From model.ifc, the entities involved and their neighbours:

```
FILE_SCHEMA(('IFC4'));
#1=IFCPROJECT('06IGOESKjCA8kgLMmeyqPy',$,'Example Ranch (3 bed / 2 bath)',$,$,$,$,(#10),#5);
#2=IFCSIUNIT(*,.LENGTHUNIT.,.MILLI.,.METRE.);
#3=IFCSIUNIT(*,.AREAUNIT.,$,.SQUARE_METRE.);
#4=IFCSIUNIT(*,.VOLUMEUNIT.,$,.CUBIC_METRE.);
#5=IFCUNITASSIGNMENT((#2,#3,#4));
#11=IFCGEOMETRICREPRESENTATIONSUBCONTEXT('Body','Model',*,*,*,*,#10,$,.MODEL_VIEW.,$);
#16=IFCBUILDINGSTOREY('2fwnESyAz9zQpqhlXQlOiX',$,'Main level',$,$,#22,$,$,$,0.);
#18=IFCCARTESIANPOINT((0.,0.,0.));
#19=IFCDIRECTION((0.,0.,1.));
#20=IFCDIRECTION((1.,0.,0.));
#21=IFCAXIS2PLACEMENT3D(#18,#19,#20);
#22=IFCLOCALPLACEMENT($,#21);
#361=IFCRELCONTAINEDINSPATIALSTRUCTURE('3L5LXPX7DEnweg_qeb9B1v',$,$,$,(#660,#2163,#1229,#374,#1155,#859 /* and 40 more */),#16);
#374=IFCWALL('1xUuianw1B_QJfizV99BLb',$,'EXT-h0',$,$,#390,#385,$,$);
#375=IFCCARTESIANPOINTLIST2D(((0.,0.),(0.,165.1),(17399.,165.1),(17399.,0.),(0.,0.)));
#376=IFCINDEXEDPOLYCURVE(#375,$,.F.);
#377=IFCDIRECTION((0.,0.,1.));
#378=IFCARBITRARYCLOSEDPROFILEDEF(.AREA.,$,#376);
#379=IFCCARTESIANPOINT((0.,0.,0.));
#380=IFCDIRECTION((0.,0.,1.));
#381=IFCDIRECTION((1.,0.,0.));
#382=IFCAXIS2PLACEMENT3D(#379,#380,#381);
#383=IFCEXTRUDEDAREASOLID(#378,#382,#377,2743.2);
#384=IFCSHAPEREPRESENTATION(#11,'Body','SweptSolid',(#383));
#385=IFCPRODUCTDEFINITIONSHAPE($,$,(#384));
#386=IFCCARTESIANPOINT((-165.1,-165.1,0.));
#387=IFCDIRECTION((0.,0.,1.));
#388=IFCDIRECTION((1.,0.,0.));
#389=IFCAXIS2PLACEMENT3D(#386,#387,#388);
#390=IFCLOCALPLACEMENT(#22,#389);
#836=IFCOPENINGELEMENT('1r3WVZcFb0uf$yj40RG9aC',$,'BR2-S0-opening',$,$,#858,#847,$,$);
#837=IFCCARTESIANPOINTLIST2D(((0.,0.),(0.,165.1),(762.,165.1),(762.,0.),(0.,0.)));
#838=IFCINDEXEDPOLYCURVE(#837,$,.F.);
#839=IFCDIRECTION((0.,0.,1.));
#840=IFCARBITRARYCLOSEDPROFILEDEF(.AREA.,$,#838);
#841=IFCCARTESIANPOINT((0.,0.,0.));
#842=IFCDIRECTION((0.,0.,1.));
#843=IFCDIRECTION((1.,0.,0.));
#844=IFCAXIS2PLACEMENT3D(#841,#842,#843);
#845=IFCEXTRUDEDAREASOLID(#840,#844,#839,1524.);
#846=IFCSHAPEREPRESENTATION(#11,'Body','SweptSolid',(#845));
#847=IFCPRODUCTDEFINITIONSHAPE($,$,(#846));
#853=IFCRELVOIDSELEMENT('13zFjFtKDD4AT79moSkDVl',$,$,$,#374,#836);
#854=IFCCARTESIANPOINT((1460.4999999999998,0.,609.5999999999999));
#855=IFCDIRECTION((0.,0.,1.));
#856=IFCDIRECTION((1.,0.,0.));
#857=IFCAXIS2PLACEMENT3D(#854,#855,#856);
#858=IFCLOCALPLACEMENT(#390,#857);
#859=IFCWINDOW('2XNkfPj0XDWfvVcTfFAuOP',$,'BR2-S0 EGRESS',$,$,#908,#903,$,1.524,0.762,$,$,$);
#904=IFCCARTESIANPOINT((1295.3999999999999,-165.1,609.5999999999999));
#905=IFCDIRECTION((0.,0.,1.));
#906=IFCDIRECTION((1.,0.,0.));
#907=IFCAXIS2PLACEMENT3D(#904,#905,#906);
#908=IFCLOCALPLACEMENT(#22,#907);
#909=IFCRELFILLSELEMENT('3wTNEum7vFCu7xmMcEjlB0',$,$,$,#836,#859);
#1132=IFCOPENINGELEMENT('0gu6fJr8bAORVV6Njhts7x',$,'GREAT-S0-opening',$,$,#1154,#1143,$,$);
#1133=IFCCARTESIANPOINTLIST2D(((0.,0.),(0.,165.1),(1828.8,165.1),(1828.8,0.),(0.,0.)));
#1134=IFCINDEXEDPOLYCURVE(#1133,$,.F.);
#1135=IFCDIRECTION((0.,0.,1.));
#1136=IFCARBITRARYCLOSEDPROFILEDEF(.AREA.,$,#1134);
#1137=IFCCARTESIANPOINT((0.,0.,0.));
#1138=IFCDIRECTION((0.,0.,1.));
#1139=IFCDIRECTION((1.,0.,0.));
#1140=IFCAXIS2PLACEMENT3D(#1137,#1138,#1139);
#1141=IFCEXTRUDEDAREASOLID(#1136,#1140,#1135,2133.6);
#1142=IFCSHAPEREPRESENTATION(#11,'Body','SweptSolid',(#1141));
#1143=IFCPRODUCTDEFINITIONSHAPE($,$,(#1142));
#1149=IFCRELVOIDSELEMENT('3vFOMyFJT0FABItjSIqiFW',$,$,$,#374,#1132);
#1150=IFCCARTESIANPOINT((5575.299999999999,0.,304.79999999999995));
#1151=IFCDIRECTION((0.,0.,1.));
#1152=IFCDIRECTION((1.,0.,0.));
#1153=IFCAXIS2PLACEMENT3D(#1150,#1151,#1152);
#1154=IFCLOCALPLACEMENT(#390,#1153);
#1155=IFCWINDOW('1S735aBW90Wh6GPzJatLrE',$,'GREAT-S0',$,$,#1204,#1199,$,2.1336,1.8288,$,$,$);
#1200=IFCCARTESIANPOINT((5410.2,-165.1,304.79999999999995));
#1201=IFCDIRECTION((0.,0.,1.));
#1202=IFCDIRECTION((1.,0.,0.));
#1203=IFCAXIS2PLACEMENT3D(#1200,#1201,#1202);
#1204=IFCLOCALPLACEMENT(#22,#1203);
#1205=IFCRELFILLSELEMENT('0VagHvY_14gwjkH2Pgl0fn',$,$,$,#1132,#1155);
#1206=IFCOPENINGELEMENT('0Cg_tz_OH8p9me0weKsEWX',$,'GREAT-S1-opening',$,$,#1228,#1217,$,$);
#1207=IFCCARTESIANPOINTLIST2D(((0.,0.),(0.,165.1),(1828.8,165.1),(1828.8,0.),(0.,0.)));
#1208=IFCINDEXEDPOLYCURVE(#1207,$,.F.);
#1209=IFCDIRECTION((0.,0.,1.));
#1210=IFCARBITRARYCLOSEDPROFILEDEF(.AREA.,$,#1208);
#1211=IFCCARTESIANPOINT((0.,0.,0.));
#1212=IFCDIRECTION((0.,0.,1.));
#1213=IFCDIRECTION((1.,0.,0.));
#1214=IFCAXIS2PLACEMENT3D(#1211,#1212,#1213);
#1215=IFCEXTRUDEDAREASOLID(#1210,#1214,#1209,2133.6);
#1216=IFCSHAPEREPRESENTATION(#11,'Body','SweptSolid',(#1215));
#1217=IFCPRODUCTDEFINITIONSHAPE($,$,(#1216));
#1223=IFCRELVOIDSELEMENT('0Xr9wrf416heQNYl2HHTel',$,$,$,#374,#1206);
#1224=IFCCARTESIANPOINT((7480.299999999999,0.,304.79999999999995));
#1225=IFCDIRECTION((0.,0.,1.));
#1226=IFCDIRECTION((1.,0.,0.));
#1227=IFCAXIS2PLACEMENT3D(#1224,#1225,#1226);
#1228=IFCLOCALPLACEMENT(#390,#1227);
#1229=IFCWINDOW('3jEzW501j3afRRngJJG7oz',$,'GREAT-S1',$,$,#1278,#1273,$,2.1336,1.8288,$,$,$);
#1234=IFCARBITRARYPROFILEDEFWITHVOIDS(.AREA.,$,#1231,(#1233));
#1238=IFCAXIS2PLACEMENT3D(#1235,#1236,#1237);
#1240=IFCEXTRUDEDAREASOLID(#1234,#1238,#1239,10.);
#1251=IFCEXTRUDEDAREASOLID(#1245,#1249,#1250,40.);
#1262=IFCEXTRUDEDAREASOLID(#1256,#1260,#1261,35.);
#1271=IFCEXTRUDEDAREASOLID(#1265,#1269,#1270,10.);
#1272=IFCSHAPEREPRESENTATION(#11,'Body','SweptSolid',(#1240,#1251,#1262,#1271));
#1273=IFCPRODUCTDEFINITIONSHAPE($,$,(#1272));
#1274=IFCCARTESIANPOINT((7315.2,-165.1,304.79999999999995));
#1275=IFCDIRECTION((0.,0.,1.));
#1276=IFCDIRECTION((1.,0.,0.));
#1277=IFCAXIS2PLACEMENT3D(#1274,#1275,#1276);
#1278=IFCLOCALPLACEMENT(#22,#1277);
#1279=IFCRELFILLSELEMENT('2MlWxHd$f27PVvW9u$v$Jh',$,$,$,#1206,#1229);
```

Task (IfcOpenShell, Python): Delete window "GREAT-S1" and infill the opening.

```python
import ifcopenshell
import ifcopenshell.api.feature
import ifcopenshell.api.root
import ifcopenshell.geom
import ifcopenshell.util.shape

model = ifcopenshell.open("model.ifc")
settings = ifcopenshell.geom.settings()


def volume(element):
    """Net volume in cubic metres, openings subtracted."""
    shape = ifcopenshell.geom.create_shape(settings, element)
    return ifcopenshell.util.shape.get_volume(shape.geometry)


window = model.by_id(1229)
opening = window.FillsVoids[0].RelatingOpeningElement
wall = opening.VoidsElements[0].RelatingBuildingElement
before = volume(wall)

ifcopenshell.api.root.remove_product(model, product=window)
ifcopenshell.api.feature.remove_feature(model, feature=opening)

after = volume(wall)

print(f"wall volume {before:.3f} -> {after:.3f} m3")

model.write("model_rev.ifc")
```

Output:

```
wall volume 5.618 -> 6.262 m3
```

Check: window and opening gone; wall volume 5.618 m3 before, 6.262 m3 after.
